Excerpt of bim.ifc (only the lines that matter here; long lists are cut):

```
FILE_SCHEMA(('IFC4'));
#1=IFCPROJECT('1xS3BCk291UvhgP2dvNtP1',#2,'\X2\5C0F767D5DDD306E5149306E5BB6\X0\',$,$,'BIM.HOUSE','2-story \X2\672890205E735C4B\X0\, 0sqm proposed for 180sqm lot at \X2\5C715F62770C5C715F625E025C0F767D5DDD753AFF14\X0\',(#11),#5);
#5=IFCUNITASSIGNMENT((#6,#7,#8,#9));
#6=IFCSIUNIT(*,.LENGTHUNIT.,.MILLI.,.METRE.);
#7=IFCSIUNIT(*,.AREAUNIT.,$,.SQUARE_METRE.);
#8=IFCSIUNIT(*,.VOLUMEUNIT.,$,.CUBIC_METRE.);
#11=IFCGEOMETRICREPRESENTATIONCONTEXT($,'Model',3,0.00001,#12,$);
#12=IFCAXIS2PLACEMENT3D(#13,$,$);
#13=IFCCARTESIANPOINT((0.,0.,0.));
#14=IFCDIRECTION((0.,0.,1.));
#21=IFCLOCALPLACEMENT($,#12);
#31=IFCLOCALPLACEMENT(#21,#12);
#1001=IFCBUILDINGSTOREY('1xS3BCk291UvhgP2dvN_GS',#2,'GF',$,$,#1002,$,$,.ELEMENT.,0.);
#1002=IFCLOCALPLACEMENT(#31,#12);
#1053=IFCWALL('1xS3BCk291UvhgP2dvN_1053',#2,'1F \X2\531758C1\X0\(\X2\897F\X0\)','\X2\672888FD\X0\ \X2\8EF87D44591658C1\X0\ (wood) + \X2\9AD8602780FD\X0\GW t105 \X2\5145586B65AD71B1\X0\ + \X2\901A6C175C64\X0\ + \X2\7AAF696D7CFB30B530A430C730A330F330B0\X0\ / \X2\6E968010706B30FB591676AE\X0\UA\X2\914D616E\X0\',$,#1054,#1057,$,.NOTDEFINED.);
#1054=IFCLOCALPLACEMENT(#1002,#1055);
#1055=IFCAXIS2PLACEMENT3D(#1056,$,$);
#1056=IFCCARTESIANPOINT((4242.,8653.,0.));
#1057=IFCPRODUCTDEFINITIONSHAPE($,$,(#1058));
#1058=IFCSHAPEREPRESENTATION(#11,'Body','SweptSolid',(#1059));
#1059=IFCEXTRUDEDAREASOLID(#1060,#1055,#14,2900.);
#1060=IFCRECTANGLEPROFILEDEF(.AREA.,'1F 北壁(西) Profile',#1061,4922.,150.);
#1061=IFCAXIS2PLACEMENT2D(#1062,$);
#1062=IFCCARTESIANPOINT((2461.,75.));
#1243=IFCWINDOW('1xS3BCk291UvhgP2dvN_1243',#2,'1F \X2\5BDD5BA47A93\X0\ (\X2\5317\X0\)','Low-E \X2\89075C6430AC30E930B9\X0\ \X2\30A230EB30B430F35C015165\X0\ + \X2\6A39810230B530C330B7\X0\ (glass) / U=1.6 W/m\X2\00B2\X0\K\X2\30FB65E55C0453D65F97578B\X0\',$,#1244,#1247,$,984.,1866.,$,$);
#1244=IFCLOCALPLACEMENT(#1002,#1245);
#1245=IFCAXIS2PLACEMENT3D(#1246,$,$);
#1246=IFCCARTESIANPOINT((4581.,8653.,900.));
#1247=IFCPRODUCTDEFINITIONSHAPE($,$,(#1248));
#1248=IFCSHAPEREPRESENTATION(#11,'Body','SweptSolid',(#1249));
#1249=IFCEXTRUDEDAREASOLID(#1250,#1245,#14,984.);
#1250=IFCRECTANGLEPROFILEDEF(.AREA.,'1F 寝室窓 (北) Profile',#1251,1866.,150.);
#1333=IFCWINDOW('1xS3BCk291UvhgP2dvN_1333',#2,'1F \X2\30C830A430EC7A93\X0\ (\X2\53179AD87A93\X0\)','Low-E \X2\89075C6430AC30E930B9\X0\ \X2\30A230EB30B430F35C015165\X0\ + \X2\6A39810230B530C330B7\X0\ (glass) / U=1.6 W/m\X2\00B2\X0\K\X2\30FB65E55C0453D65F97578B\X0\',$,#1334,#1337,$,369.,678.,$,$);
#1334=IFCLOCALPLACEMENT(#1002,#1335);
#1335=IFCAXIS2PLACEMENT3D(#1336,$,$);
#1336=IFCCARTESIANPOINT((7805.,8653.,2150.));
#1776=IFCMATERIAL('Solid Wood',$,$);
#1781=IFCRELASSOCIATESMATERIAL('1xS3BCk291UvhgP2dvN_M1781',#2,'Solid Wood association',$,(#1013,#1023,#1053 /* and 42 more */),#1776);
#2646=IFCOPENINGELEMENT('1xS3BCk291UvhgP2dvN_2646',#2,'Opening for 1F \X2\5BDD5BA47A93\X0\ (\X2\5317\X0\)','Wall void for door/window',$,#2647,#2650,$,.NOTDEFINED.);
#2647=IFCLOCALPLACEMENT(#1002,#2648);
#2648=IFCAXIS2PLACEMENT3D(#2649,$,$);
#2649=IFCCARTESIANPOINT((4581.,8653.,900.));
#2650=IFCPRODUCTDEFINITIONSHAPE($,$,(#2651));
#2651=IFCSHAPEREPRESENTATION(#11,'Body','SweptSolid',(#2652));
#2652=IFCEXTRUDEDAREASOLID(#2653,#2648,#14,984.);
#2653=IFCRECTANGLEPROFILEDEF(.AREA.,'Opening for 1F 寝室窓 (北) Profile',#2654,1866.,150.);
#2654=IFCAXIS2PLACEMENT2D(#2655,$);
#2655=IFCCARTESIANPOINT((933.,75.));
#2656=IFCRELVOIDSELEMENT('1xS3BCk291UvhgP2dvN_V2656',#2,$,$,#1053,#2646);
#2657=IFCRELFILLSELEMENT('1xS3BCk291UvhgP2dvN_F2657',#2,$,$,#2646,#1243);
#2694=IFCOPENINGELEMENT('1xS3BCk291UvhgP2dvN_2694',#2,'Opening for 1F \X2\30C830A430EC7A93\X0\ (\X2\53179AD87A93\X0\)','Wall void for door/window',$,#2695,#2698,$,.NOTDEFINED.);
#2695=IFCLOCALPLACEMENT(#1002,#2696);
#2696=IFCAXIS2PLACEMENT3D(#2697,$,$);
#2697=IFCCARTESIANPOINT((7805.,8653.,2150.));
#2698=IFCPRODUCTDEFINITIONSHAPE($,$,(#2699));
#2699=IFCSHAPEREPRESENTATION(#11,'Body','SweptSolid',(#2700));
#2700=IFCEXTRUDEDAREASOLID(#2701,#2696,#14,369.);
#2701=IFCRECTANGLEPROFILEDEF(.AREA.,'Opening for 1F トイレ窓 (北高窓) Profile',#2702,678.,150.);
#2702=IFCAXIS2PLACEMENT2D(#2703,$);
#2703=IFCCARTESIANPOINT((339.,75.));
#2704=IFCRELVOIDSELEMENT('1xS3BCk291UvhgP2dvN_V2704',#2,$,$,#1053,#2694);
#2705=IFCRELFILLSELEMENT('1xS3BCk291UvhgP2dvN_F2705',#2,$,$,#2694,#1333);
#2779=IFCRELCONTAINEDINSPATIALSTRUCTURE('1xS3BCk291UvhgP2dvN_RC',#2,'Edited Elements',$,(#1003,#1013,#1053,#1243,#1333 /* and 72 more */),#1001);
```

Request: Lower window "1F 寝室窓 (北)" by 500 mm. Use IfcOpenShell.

```python
import numpy as np
import ifcopenshell
import ifcopenshell.api.geometry
import ifcopenshell.util.placement
import ifcopenshell.util.unit

model = ifcopenshell.open("bim.ifc")
unit_scale = ifcopenshell.util.unit.calculate_unit_scale(model)

window = model.by_guid("1xS3BCk291UvhgP2dvN_1243")
opening = window.FillsVoids[0].RelatingOpeningElement
dz = -0.5 / unit_scale

shift = np.array([0.0, 0.0, dz])
# The window is not placed relative to its opening, so move both.
for product in (opening, window):
    matrix = ifcopenshell.util.placement.get_local_placement(product.ObjectPlacement)
    matrix[:3, 3] += shift
    ifcopenshell.api.geometry.edit_object_placement(model, product=product, matrix=matrix, is_si=False)

print(f"moved by {dz * unit_scale:+.3f} m")

model.write("bim_edited.ifc")
```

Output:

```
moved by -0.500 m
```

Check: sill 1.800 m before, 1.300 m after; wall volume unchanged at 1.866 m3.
